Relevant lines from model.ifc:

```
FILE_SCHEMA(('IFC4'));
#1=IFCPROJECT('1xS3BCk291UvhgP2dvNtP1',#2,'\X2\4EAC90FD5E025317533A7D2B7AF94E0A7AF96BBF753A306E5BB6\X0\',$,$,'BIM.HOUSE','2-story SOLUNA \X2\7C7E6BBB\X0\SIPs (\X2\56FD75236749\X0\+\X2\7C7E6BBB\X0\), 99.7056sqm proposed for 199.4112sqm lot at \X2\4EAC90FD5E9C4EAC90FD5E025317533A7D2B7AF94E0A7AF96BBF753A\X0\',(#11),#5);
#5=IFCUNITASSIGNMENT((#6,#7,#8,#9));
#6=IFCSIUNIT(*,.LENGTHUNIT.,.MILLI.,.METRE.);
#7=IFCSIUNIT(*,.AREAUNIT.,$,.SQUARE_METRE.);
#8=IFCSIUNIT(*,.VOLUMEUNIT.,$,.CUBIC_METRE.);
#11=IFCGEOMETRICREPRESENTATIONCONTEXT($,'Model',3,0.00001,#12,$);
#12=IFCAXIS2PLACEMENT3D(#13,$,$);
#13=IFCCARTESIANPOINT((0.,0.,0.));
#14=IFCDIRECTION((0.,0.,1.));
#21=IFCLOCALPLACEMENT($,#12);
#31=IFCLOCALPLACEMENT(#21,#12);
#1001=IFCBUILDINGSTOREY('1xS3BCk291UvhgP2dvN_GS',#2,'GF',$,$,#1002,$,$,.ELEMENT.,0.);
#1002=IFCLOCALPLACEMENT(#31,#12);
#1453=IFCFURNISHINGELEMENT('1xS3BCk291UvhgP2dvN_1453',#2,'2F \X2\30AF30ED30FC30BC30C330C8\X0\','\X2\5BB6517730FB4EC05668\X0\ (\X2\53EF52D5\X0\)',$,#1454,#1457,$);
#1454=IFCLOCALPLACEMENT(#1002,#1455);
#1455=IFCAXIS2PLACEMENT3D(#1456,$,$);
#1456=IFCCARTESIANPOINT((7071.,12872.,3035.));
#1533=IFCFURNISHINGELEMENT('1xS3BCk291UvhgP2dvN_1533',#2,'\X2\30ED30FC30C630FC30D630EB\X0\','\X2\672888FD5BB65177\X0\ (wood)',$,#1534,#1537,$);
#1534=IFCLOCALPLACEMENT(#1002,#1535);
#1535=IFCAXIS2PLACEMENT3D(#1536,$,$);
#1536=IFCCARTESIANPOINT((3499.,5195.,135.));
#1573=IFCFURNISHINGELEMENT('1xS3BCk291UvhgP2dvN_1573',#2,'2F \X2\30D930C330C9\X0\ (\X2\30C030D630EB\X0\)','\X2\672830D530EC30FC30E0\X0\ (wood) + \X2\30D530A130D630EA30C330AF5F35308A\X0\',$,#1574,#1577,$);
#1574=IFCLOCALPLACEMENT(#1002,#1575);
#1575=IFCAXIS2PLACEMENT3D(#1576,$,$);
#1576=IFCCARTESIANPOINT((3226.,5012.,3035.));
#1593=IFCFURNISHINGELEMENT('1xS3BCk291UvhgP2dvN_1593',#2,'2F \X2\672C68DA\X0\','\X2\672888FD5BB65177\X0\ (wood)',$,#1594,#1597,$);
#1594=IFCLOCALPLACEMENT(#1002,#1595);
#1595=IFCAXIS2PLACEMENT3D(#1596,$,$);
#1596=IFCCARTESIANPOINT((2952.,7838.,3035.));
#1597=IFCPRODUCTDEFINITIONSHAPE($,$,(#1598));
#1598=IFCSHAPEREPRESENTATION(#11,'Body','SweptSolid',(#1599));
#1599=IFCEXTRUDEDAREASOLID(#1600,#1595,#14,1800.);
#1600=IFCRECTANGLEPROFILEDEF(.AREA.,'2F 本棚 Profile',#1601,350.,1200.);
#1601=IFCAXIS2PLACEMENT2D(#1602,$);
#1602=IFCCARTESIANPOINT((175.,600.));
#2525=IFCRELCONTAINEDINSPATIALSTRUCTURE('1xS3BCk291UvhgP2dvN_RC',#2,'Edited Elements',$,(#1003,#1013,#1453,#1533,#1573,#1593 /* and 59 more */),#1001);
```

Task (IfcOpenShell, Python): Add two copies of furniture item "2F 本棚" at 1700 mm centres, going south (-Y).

```python
import numpy as np
import ifcopenshell
import ifcopenshell.api.geometry
import ifcopenshell.api.root
import ifcopenshell.util.element
import ifcopenshell.util.placement
import ifcopenshell.util.unit

model = ifcopenshell.open("model.ifc")
unit_scale = ifcopenshell.util.unit.calculate_unit_scale(model)


def reuse_history(source, copy):
    """copy_class also copies each property set's owner history, people and application; keep the originals."""
    for rel in copy.IsDefinedBy:
        if rel.is_a("IfcRelDefinesByProperties") and (history := rel.RelatingPropertyDefinition.OwnerHistory):
            rel.RelatingPropertyDefinition.OwnerHistory = source.OwnerHistory
            ifcopenshell.util.element.remove_deep2(model, history)


source = model.by_id(1593)
base = ifcopenshell.util.placement.get_local_placement(source.ObjectPlacement)
step = np.array([0.0, -1.0, 0.0]) * 1.7 / unit_scale

for i in range(1, 3):
    copy = ifcopenshell.api.root.copy_class(model, product=source)
    copy.Representation = ifcopenshell.util.element.copy_deep(
        model, source.Representation, exclude=["IfcGeometricRepresentationContext", "IfcRepresentationMap"]
    )
    reuse_history(source, copy)
    matrix = base.copy()
    matrix[:3, 3] += i * step
    print("added at", matrix[:3, 3].round(3) + 0.0)
    ifcopenshell.api.geometry.edit_object_placement(model, product=copy, matrix=matrix, is_si=False)

model.write("model_v2.ifc")
```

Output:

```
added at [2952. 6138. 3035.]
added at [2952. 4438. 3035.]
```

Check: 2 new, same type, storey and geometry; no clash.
